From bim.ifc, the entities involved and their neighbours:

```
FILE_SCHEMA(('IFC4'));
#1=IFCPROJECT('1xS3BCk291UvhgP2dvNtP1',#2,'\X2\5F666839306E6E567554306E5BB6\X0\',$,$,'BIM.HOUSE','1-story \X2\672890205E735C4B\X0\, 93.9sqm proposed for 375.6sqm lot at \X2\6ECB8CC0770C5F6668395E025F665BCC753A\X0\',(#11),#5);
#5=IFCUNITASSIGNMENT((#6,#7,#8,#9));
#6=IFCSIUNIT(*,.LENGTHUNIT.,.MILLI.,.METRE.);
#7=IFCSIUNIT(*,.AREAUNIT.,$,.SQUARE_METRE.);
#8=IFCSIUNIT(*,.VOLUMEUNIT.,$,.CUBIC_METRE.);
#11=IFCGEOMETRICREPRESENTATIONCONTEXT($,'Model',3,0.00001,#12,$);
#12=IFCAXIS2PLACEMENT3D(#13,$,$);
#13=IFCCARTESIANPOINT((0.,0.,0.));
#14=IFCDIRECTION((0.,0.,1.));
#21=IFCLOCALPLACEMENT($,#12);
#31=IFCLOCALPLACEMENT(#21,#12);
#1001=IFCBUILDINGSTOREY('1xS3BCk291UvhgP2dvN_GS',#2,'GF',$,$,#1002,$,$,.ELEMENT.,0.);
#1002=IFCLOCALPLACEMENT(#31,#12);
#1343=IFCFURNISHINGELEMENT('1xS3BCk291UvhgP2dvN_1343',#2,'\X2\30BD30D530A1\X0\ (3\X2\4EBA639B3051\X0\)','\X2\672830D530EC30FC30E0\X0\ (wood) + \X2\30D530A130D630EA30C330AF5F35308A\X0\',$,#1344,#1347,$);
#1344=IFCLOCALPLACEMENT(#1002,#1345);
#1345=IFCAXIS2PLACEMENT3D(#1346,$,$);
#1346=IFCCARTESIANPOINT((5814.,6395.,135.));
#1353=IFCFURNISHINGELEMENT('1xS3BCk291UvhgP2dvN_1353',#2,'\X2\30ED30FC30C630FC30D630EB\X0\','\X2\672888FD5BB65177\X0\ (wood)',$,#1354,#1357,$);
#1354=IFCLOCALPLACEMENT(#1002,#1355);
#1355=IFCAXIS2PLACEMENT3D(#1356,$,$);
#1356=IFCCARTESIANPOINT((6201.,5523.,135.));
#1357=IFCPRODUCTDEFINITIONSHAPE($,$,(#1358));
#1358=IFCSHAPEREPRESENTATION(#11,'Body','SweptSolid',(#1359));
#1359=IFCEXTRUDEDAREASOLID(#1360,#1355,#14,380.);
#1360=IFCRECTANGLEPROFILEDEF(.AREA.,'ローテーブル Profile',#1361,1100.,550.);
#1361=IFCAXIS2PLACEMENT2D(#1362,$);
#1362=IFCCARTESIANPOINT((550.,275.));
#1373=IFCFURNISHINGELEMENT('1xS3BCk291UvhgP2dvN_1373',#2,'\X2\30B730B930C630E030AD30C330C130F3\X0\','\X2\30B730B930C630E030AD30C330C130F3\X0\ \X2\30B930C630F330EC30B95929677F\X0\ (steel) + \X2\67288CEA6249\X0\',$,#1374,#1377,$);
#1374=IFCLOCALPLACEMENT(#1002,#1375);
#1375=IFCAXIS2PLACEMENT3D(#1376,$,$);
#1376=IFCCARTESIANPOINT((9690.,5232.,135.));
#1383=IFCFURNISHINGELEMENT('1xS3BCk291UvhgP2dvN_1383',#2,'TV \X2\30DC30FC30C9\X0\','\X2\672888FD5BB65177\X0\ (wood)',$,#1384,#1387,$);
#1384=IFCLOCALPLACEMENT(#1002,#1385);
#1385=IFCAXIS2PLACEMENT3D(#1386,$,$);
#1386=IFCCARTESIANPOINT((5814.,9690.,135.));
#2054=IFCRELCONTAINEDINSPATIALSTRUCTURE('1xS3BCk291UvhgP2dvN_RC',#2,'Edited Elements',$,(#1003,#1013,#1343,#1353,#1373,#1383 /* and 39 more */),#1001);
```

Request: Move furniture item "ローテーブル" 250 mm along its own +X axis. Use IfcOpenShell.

```python
import ifcopenshell
import ifcopenshell.api.geometry
import ifcopenshell.util.placement
import ifcopenshell.util.unit

model = ifcopenshell.open("bim.ifc")
unit_scale = ifcopenshell.util.unit.calculate_unit_scale(model)

item = model.by_guid("1xS3BCk291UvhgP2dvN_1353")
matrix = ifcopenshell.util.placement.get_local_placement(item.ObjectPlacement)
matrix[:3, 3] += matrix[:3, 0] * 0.25 / unit_scale
ifcopenshell.api.geometry.edit_object_placement(model, product=item, matrix=matrix, is_si=False)

print(ifcopenshell.util.placement.get_local_placement(item.ObjectPlacement).round(3) + 0.0)

model.write("bim_rev.ifc")
```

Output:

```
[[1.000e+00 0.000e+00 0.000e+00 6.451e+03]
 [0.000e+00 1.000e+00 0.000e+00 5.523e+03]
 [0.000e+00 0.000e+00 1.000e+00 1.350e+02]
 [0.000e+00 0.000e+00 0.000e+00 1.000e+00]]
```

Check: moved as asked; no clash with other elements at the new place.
